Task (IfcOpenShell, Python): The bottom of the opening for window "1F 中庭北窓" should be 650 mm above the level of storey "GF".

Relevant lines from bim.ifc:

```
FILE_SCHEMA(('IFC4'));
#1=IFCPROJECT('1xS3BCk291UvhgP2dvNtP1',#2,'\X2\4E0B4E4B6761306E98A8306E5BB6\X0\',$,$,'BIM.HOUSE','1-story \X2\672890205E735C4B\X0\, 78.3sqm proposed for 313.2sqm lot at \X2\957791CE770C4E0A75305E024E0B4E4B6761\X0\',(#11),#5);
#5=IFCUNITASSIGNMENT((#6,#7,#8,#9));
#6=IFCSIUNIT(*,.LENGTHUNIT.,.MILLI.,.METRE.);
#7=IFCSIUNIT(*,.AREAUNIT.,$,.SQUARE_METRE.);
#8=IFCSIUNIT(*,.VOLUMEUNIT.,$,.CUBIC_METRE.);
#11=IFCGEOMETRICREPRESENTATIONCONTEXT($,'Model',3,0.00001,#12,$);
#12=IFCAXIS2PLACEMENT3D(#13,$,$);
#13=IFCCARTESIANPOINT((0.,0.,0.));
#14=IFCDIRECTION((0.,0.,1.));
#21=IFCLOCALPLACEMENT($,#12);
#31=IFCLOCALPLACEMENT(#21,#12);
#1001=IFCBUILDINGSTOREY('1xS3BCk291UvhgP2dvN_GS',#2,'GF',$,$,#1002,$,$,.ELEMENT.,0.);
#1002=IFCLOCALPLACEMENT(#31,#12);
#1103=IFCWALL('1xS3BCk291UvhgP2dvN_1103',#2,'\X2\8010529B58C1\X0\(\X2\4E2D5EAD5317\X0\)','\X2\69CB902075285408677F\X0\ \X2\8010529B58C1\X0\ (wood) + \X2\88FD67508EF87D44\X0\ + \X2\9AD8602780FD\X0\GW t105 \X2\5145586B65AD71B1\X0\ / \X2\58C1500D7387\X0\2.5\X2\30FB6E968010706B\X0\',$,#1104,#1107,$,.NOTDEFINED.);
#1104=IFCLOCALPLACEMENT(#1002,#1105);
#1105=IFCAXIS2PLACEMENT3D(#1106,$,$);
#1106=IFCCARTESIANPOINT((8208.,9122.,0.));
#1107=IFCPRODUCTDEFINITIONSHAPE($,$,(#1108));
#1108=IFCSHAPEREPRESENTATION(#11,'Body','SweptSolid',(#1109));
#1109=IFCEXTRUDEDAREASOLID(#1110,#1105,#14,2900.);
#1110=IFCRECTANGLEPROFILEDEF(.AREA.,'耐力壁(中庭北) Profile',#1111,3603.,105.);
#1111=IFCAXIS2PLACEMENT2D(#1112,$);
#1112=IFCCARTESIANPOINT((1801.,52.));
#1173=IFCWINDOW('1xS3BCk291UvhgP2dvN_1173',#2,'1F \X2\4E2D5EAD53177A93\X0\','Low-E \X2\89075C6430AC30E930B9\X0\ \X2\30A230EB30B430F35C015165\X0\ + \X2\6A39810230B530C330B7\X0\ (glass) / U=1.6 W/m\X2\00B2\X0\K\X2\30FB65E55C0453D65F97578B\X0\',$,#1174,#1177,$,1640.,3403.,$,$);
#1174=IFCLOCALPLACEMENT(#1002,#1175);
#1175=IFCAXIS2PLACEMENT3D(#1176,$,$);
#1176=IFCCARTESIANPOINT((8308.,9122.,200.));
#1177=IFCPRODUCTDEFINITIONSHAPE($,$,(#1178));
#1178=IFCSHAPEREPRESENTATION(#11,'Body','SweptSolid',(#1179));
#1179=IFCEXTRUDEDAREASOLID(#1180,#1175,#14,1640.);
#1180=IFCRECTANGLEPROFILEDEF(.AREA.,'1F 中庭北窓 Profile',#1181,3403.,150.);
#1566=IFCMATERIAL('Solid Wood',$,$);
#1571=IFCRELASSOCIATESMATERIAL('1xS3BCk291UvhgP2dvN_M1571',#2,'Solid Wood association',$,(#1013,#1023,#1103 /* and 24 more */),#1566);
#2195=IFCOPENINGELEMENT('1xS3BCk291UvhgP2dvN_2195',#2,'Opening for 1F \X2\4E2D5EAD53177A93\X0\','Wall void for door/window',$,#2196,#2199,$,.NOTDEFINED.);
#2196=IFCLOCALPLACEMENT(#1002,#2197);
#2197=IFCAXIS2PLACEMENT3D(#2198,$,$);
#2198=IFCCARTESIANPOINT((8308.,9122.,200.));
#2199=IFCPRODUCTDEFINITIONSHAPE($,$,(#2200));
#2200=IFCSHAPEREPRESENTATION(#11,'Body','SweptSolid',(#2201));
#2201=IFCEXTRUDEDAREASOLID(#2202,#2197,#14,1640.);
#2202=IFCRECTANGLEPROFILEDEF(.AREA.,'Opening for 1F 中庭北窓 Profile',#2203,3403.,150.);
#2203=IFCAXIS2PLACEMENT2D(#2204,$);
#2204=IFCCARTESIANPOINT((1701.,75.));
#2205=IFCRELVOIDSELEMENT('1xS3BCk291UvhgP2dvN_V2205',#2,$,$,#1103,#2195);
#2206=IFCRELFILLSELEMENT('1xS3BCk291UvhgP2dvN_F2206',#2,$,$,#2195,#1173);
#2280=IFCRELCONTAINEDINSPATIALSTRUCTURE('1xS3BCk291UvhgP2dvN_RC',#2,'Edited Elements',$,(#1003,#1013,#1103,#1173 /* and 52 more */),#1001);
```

```python
import numpy as np
import ifcopenshell
import ifcopenshell.api.geometry
import ifcopenshell.geom
import ifcopenshell.util.element
import ifcopenshell.util.placement
import ifcopenshell.util.shape
import ifcopenshell.util.unit

model = ifcopenshell.open("bim.ifc")
unit_scale = ifcopenshell.util.unit.calculate_unit_scale(model)

window = model.by_id(1173)
opening = window.FillsVoids[0].RelatingOpeningElement
storey = ifcopenshell.util.element.get_container(window, ifc_class="IfcBuildingStorey")
level = ifcopenshell.util.placement.get_local_placement(storey.ObjectPlacement)[2, 3]

# The opening's origin need not be at the sill, so measure its lowest point.
shape = ifcopenshell.geom.create_shape(ifcopenshell.geom.settings(), opening)
bottom = ifcopenshell.util.shape.get_shape_bottom_elevation(shape, shape.geometry) / unit_scale
dz = level + 650.0 - bottom

shift = np.array([0.0, 0.0, dz])
# The window is not placed relative to its opening, so move both.
for product in (opening, window):
    matrix = ifcopenshell.util.placement.get_local_placement(product.ObjectPlacement)
    matrix[:3, 3] += shift
    ifcopenshell.api.geometry.edit_object_placement(model, product=product, matrix=matrix, is_si=False)

print(f"moved by {dz * unit_scale:+.3f} m")

model.write("bim_updated.ifc")
```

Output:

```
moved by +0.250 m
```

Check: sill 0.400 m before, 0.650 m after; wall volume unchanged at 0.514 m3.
